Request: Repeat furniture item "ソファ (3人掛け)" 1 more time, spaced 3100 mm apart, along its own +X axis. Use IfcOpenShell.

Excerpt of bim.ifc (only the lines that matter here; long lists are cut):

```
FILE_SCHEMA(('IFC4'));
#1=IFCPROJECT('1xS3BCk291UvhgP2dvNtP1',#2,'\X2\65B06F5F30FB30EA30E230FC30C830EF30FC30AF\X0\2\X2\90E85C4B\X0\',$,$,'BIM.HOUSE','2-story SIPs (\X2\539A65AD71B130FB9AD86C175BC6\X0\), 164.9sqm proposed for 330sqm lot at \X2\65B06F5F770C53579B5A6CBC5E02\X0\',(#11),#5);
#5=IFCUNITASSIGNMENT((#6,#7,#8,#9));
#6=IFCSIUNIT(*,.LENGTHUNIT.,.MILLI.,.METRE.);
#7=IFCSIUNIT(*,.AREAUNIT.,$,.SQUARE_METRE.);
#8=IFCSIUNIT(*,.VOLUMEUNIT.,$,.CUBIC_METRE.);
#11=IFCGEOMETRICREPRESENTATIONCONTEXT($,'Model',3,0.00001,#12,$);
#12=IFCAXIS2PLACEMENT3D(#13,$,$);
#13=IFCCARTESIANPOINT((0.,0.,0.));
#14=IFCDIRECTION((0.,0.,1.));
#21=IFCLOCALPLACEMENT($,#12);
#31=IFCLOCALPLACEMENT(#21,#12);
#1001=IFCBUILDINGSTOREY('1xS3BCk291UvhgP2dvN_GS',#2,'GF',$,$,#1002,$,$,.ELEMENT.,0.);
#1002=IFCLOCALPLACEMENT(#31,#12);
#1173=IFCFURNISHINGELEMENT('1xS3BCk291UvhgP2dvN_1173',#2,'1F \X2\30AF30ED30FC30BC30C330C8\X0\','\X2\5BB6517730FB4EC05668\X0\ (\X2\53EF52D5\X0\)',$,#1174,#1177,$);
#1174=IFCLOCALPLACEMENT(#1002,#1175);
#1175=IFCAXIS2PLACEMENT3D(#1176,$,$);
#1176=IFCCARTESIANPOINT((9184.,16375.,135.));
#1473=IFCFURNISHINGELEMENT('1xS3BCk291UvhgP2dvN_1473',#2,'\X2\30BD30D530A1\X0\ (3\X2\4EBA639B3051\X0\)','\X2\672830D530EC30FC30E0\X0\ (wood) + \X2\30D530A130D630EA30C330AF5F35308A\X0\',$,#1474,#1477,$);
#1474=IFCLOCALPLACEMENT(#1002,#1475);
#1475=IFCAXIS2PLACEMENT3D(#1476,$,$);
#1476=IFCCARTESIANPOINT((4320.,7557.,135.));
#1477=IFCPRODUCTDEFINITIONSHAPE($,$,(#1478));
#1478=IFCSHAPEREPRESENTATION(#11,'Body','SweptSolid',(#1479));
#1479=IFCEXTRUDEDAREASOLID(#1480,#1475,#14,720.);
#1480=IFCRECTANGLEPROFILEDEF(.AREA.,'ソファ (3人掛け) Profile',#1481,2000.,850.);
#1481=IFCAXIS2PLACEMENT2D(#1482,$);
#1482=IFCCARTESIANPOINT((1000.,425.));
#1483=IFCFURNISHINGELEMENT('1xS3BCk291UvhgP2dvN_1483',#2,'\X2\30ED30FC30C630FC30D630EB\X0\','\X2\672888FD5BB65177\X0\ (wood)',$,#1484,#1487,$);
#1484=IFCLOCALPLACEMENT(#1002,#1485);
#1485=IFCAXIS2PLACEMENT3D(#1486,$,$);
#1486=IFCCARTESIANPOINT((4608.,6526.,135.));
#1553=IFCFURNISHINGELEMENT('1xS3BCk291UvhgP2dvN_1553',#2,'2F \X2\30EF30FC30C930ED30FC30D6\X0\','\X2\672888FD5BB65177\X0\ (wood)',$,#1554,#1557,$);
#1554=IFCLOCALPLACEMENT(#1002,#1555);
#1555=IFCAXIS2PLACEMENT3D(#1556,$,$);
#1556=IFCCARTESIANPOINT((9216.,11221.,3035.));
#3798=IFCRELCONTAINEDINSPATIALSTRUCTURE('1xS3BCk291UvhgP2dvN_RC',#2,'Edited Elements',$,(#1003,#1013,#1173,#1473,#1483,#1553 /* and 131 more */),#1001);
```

```python
import ifcopenshell
import ifcopenshell.api.geometry
import ifcopenshell.api.root
import ifcopenshell.util.element
import ifcopenshell.util.placement
import ifcopenshell.util.unit

model = ifcopenshell.open("bim.ifc")
unit_scale = ifcopenshell.util.unit.calculate_unit_scale(model)


def reuse_history(source, copy):
    """copy_class also copies each property set's owner history, people and application; keep the originals."""
    for rel in copy.IsDefinedBy:
        if rel.is_a("IfcRelDefinesByProperties") and (history := rel.RelatingPropertyDefinition.OwnerHistory):
            rel.RelatingPropertyDefinition.OwnerHistory = source.OwnerHistory
            ifcopenshell.util.element.remove_deep2(model, history)


source = model.by_id(1473)
base = ifcopenshell.util.placement.get_local_placement(source.ObjectPlacement)
step = base[:3, 0] * 3.1 / unit_scale

for i in range(1, 2):
    copy = ifcopenshell.api.root.copy_class(model, product=source)
    copy.Representation = ifcopenshell.util.element.copy_deep(
        model, source.Representation, exclude=["IfcGeometricRepresentationContext", "IfcRepresentationMap"]
    )
    reuse_history(source, copy)
    matrix = base.copy()
    matrix[:3, 3] += i * step
    print("added at", matrix[:3, 3].round(3) + 0.0)
    ifcopenshell.api.geometry.edit_object_placement(model, product=copy, matrix=matrix, is_si=False)

model.write("bim_v2.ifc")
```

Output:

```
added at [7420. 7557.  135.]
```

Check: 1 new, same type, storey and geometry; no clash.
